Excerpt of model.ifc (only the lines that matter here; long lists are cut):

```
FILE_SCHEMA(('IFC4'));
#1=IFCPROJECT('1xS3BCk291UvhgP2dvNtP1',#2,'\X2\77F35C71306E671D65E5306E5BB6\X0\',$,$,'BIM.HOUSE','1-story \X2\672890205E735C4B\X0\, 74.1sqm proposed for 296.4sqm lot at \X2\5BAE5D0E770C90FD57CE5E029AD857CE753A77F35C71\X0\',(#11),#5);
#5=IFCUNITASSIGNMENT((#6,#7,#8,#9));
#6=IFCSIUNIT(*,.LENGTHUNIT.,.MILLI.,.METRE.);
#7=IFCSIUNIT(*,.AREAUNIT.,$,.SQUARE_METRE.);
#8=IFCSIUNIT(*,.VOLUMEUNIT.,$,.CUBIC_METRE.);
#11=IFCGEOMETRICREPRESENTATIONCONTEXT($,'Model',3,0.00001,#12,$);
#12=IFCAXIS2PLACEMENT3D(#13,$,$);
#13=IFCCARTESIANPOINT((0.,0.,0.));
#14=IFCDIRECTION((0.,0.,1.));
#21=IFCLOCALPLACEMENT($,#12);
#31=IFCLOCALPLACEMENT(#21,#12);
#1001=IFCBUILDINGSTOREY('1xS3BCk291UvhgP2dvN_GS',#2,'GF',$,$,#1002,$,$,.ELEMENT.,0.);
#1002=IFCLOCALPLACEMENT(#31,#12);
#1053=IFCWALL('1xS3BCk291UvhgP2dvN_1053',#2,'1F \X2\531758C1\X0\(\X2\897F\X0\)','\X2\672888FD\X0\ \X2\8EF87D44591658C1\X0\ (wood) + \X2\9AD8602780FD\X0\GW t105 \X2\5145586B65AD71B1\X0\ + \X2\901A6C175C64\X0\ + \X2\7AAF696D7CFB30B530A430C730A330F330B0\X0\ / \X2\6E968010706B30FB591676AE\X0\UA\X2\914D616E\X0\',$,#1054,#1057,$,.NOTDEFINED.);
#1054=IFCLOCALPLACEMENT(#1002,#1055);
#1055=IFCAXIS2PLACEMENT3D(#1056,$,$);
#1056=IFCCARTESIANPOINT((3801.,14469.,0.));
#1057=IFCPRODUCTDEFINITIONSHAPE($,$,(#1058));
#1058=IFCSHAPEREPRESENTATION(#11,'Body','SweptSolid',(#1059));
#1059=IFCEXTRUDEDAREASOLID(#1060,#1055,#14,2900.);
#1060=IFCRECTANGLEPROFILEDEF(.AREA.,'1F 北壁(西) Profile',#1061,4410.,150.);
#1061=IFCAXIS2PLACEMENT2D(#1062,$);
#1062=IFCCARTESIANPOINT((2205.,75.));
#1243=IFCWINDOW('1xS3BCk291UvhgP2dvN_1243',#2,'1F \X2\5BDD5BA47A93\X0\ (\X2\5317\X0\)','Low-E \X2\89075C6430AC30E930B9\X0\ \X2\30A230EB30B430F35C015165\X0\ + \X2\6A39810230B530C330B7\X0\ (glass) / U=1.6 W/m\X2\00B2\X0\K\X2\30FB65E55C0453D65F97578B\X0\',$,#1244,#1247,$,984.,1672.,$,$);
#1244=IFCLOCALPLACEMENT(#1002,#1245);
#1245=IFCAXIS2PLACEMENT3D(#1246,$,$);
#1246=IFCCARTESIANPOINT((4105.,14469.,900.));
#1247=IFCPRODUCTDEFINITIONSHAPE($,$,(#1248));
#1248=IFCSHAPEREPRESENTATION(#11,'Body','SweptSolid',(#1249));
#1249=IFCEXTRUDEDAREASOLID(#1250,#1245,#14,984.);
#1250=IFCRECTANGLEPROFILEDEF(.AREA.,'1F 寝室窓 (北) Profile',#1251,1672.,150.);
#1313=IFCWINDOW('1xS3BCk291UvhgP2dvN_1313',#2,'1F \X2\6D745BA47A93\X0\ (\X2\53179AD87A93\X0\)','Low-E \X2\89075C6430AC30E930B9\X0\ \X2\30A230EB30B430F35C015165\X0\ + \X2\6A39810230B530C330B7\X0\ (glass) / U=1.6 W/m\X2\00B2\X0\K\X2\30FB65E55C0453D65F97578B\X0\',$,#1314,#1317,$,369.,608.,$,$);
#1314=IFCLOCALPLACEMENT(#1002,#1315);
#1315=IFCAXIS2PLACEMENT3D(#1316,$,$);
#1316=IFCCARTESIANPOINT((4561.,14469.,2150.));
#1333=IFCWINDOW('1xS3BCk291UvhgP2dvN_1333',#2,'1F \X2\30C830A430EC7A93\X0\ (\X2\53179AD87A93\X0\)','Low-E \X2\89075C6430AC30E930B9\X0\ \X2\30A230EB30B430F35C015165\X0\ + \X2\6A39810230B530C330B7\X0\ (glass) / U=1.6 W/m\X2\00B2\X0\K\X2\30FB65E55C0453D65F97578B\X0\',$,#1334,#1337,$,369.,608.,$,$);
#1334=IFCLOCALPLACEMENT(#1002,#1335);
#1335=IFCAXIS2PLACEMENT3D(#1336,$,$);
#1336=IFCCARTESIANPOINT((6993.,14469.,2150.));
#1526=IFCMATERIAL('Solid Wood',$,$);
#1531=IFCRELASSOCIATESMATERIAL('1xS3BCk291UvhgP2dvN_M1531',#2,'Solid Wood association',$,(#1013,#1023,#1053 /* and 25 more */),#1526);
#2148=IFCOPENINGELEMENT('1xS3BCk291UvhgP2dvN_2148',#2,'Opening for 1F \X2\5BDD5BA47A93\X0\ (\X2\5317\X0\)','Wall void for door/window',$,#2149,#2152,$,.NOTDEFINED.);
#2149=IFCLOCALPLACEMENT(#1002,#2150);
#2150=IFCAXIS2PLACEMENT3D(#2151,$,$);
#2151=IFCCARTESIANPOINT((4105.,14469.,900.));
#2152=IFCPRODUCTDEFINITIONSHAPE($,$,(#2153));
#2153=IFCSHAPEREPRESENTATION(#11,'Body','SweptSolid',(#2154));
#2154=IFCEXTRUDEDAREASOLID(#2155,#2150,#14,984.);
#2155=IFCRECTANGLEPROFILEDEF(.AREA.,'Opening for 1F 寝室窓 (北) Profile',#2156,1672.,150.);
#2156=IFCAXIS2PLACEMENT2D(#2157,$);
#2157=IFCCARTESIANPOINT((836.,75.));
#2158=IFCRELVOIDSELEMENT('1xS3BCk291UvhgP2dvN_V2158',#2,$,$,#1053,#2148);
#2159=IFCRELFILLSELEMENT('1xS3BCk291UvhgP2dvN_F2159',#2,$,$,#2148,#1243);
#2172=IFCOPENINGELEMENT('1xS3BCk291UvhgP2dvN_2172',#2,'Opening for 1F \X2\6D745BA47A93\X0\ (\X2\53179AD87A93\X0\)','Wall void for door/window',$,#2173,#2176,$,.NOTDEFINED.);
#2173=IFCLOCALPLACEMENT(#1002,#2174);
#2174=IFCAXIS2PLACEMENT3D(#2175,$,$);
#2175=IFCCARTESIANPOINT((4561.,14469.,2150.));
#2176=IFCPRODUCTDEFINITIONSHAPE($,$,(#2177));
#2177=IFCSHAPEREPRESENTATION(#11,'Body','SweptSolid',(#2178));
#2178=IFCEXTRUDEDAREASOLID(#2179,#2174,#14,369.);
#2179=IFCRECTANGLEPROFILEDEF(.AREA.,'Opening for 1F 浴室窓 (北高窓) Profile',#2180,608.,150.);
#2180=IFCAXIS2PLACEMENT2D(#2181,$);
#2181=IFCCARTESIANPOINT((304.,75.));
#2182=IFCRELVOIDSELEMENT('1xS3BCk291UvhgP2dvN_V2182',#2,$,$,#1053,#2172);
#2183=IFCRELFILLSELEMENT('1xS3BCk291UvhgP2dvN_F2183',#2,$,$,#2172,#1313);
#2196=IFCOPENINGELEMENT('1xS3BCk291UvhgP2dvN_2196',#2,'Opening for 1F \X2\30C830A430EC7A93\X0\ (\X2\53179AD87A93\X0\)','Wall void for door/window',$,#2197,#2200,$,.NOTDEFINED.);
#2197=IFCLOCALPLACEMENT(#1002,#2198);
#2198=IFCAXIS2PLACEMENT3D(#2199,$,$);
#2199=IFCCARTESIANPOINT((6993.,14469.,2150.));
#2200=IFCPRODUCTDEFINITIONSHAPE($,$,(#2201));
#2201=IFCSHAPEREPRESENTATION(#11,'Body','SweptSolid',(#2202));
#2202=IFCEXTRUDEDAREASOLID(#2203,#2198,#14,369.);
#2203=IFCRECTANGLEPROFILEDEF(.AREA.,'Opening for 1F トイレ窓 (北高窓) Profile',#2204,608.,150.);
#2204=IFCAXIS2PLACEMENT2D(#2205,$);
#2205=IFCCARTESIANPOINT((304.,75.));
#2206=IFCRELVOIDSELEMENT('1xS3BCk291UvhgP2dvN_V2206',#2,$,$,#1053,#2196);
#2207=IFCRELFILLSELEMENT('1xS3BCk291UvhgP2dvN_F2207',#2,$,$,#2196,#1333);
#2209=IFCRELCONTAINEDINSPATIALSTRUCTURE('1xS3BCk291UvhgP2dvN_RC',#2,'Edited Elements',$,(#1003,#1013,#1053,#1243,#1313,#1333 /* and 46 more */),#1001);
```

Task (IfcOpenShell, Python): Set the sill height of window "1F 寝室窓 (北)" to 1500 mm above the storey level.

```python
import numpy as np
import ifcopenshell
import ifcopenshell.api.geometry
import ifcopenshell.geom
import ifcopenshell.util.element
import ifcopenshell.util.placement
import ifcopenshell.util.shape
import ifcopenshell.util.unit

model = ifcopenshell.open("model.ifc")
unit_scale = ifcopenshell.util.unit.calculate_unit_scale(model)

window = model.by_guid("1xS3BCk291UvhgP2dvN_1243")
opening = window.FillsVoids[0].RelatingOpeningElement
storey = ifcopenshell.util.element.get_container(window, ifc_class="IfcBuildingStorey")
level = ifcopenshell.util.placement.get_local_placement(storey.ObjectPlacement)[2, 3]

# The opening's origin need not be at the sill, so measure its lowest point.
shape = ifcopenshell.geom.create_shape(ifcopenshell.geom.settings(), opening)
bottom = ifcopenshell.util.shape.get_shape_bottom_elevation(shape, shape.geometry) / unit_scale
dz = level + 1500.0 - bottom

shift = np.array([0.0, 0.0, dz])
# The window is not placed relative to its opening, so move both.
for product in (opening, window):
    matrix = ifcopenshell.util.placement.get_local_placement(product.ObjectPlacement)
    matrix[:3, 3] += shift
    ifcopenshell.api.geometry.edit_object_placement(model, product=product, matrix=matrix, is_si=False)

print(f"moved by {dz * unit_scale:+.3f} m")

model.write("model_rev.ifc")
```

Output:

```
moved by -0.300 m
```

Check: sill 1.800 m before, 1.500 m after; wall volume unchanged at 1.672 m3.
